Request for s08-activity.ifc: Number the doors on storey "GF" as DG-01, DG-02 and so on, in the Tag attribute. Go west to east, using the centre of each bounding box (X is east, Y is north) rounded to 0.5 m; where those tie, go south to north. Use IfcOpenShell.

First a look at what the model holds.

```python
import ifcopenshell
import ifcopenshell.util.element
import ifcopenshell.util.placement

model = ifcopenshell.open("s08-activity.ifc")
print(model.schema)
storey = next(s for s in model.by_type("IfcBuildingStorey") if s.Name == "GF")
doors = [e for e in ifcopenshell.util.element.get_decomposition(storey) if e.is_a("IfcDoor")]
for e in sorted(doors, key=lambda e: e.id()):
    origin = ifcopenshell.util.placement.get_local_placement(e.ObjectPlacement)[:3, 3]
    print(e.id(), e.Tag, e.Name, origin.round(2) + 0.0, sep=" | ")
```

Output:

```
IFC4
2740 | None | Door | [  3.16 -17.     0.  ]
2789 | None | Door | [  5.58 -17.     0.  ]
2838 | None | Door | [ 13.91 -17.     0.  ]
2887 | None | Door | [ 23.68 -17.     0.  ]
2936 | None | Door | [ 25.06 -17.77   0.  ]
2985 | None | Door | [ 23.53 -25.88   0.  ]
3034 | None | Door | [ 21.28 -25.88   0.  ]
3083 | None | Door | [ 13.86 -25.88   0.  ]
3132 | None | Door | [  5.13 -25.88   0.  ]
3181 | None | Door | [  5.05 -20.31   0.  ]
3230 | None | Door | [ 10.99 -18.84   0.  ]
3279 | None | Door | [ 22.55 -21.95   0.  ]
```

```python
import ifcopenshell
import ifcopenshell.geom
import ifcopenshell.util.element
import ifcopenshell.util.shape

model = ifcopenshell.open("s08-activity.ifc")
settings = ifcopenshell.geom.settings()
settings.set("use-world-coords", True)


def centre(element):
    shape = ifcopenshell.geom.create_shape(settings, element)
    return ifcopenshell.util.shape.get_bbox_centroid(shape.geometry)


storey = next(s for s in model.by_type("IfcBuildingStorey") if s.Name == "GF")
doors = [e for e in ifcopenshell.util.element.get_decomposition(storey) if e.is_a("IfcDoor")]

# Insertion points can sit at a corner or the storey origin, so sort by the geometry (in metres).
centres = {e: centre(e) for e in doors}
doors.sort(key=lambda e: (round(centres[e][0] / 0.5), centres[e][1]))

for i, e in enumerate(doors, start=1):
    number = f"DG-{i:02d}"
    e.Tag = number
    print(e.id(), number)

model.write("s08-activity_edited.ifc")
```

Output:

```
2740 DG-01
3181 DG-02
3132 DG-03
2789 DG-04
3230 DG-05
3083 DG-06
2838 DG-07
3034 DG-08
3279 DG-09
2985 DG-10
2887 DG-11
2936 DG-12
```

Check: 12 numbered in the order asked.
